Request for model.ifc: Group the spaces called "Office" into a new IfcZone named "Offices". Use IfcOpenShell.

First a look at what the model holds.

```python
import ifcopenshell

model = ifcopenshell.open("model.ifc")
print(model.schema)
seen = {}
for space in model.by_type("IfcSpace"):
    seen[space.LongName] = seen.get(space.LongName, 0) + 1
for name, count in sorted(seen.items(), key=str):
    print(count, "x", name)
print("zones:", [z.Name for z in model.by_type("IfcZone")][:20])
```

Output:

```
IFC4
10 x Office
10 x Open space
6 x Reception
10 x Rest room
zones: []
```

```python
import ifcopenshell
import ifcopenshell.api.group
import ifcopenshell.api.root

model = ifcopenshell.open("model.ifc")

names = {"Office"}
spaces = [s for s in model.by_type("IfcSpace") if s.LongName in names]

zone = ifcopenshell.api.root.create_entity(model, ifc_class="IfcZone", name="Offices")
ifcopenshell.api.group.assign_group(model, products=spaces, group=zone)
print(len(spaces), "spaces in", zone.Name)

model.write("model_v2.ifc")
```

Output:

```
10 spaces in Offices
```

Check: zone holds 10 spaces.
